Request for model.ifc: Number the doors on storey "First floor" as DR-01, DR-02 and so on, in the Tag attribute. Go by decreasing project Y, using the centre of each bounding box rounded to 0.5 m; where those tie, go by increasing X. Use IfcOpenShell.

First a look at what the model holds.

```python
import ifcopenshell
import ifcopenshell.util.element
import ifcopenshell.util.placement

model = ifcopenshell.open("model.ifc")
print(model.schema)
storey = next(s for s in model.by_type("IfcBuildingStorey") if s.Name == "First floor")
doors = [e for e in ifcopenshell.util.element.get_decomposition(storey) if e.is_a("IfcDoor")]
for e in sorted(doors, key=lambda e: e.id()):
    origin = ifcopenshell.util.placement.get_local_placement(e.ObjectPlacement)[:3, 3]
    print(e.id(), e.Tag, e.Name, origin.round(2) + 0.0, sep=" | ")
```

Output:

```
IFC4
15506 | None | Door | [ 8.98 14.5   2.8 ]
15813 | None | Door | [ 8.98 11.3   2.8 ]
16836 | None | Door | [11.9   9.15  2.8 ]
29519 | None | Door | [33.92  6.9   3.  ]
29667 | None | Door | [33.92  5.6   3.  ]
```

```python
import ifcopenshell
import ifcopenshell.geom
import ifcopenshell.util.element
import ifcopenshell.util.shape

model = ifcopenshell.open("model.ifc")
settings = ifcopenshell.geom.settings()
settings.set("use-world-coords", True)


def centre(element):
    shape = ifcopenshell.geom.create_shape(settings, element)
    return ifcopenshell.util.shape.get_bbox_centroid(shape.geometry)


storey = next(s for s in model.by_type("IfcBuildingStorey") if s.Name == "First floor")
doors = [e for e in ifcopenshell.util.element.get_decomposition(storey) if e.is_a("IfcDoor")]

# Insertion points can sit at a corner or the storey origin, so sort by the geometry (in metres).
centres = {e: centre(e) for e in doors}
doors.sort(key=lambda e: (-round(centres[e][1] / 0.5), centres[e][0]))

for i, e in enumerate(doors, start=1):
    number = f"DR-{i:02d}"
    e.Tag = number
    print(e.id(), number)

model.write("model-out.ifc")
```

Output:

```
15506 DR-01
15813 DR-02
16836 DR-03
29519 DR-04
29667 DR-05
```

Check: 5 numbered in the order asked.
